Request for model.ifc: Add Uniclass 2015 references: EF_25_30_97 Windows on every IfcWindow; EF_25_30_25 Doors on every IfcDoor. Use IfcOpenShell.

First a look at what the model holds.

```python
import ifcopenshell

model = ifcopenshell.open("model.ifc")
print(model.schema)
print("classifications:", [c.Name for c in model.by_type("IfcClassification")])
for ifc_class in ("IfcDoor", "IfcRoof", "IfcStair", "IfcWall", "IfcWindow"):
    print(ifc_class, len(model.by_type(ifc_class)))
```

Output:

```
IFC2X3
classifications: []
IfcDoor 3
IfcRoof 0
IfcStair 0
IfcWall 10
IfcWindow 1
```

```python
import ifcopenshell
import ifcopenshell.api.classification

model = ifcopenshell.open("model.ifc")

# IFC2X3 requires Source and Edition and has no link from the project to the system.
system = model.create_entity("IfcClassification", Source="NBS", Edition="2015", Name="Uniclass 2015")

codes = {
    "IfcWindow": ("EF_25_30_97", "Windows"),
    "IfcDoor": ("EF_25_30_25", "Doors"),
}
for ifc_class, (code, name) in codes.items():
    products = model.by_type(ifc_class)
    ifcopenshell.api.classification.add_reference(
        model, products=products, classification=system, identification=code, name=name
    )
    print(code, len(products))

model.write("model_rev.ifc")
```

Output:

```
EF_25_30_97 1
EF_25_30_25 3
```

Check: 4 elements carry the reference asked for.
